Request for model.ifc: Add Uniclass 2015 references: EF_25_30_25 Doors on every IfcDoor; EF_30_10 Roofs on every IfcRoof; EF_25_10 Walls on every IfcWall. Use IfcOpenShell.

First a look at what the model holds.

```python
import ifcopenshell

model = ifcopenshell.open("model.ifc")
print(model.schema)
print("classifications:", [c.Name for c in model.by_type("IfcClassification")])
for ifc_class in ("IfcDoor", "IfcRoof", "IfcStair", "IfcWall", "IfcWindow"):
    print(ifc_class, len(model.by_type(ifc_class)))
```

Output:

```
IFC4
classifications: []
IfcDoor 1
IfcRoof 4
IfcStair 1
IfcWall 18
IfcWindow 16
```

```python
import ifcopenshell
import ifcopenshell.api.classification

model = ifcopenshell.open("model.ifc")

system = ifcopenshell.api.classification.add_classification(model, classification="Uniclass 2015")

codes = {
    "IfcDoor": ("EF_25_30_25", "Doors"),
    "IfcRoof": ("EF_30_10", "Roofs"),
    "IfcWall": ("EF_25_10", "Walls"),
}
for ifc_class, (code, name) in codes.items():
    products = model.by_type(ifc_class)
    ifcopenshell.api.classification.add_reference(
        model, products=products, classification=system, identification=code, name=name
    )
    print(code, len(products))

model.write("model_v2.ifc")
```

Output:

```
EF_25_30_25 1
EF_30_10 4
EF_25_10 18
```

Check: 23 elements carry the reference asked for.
